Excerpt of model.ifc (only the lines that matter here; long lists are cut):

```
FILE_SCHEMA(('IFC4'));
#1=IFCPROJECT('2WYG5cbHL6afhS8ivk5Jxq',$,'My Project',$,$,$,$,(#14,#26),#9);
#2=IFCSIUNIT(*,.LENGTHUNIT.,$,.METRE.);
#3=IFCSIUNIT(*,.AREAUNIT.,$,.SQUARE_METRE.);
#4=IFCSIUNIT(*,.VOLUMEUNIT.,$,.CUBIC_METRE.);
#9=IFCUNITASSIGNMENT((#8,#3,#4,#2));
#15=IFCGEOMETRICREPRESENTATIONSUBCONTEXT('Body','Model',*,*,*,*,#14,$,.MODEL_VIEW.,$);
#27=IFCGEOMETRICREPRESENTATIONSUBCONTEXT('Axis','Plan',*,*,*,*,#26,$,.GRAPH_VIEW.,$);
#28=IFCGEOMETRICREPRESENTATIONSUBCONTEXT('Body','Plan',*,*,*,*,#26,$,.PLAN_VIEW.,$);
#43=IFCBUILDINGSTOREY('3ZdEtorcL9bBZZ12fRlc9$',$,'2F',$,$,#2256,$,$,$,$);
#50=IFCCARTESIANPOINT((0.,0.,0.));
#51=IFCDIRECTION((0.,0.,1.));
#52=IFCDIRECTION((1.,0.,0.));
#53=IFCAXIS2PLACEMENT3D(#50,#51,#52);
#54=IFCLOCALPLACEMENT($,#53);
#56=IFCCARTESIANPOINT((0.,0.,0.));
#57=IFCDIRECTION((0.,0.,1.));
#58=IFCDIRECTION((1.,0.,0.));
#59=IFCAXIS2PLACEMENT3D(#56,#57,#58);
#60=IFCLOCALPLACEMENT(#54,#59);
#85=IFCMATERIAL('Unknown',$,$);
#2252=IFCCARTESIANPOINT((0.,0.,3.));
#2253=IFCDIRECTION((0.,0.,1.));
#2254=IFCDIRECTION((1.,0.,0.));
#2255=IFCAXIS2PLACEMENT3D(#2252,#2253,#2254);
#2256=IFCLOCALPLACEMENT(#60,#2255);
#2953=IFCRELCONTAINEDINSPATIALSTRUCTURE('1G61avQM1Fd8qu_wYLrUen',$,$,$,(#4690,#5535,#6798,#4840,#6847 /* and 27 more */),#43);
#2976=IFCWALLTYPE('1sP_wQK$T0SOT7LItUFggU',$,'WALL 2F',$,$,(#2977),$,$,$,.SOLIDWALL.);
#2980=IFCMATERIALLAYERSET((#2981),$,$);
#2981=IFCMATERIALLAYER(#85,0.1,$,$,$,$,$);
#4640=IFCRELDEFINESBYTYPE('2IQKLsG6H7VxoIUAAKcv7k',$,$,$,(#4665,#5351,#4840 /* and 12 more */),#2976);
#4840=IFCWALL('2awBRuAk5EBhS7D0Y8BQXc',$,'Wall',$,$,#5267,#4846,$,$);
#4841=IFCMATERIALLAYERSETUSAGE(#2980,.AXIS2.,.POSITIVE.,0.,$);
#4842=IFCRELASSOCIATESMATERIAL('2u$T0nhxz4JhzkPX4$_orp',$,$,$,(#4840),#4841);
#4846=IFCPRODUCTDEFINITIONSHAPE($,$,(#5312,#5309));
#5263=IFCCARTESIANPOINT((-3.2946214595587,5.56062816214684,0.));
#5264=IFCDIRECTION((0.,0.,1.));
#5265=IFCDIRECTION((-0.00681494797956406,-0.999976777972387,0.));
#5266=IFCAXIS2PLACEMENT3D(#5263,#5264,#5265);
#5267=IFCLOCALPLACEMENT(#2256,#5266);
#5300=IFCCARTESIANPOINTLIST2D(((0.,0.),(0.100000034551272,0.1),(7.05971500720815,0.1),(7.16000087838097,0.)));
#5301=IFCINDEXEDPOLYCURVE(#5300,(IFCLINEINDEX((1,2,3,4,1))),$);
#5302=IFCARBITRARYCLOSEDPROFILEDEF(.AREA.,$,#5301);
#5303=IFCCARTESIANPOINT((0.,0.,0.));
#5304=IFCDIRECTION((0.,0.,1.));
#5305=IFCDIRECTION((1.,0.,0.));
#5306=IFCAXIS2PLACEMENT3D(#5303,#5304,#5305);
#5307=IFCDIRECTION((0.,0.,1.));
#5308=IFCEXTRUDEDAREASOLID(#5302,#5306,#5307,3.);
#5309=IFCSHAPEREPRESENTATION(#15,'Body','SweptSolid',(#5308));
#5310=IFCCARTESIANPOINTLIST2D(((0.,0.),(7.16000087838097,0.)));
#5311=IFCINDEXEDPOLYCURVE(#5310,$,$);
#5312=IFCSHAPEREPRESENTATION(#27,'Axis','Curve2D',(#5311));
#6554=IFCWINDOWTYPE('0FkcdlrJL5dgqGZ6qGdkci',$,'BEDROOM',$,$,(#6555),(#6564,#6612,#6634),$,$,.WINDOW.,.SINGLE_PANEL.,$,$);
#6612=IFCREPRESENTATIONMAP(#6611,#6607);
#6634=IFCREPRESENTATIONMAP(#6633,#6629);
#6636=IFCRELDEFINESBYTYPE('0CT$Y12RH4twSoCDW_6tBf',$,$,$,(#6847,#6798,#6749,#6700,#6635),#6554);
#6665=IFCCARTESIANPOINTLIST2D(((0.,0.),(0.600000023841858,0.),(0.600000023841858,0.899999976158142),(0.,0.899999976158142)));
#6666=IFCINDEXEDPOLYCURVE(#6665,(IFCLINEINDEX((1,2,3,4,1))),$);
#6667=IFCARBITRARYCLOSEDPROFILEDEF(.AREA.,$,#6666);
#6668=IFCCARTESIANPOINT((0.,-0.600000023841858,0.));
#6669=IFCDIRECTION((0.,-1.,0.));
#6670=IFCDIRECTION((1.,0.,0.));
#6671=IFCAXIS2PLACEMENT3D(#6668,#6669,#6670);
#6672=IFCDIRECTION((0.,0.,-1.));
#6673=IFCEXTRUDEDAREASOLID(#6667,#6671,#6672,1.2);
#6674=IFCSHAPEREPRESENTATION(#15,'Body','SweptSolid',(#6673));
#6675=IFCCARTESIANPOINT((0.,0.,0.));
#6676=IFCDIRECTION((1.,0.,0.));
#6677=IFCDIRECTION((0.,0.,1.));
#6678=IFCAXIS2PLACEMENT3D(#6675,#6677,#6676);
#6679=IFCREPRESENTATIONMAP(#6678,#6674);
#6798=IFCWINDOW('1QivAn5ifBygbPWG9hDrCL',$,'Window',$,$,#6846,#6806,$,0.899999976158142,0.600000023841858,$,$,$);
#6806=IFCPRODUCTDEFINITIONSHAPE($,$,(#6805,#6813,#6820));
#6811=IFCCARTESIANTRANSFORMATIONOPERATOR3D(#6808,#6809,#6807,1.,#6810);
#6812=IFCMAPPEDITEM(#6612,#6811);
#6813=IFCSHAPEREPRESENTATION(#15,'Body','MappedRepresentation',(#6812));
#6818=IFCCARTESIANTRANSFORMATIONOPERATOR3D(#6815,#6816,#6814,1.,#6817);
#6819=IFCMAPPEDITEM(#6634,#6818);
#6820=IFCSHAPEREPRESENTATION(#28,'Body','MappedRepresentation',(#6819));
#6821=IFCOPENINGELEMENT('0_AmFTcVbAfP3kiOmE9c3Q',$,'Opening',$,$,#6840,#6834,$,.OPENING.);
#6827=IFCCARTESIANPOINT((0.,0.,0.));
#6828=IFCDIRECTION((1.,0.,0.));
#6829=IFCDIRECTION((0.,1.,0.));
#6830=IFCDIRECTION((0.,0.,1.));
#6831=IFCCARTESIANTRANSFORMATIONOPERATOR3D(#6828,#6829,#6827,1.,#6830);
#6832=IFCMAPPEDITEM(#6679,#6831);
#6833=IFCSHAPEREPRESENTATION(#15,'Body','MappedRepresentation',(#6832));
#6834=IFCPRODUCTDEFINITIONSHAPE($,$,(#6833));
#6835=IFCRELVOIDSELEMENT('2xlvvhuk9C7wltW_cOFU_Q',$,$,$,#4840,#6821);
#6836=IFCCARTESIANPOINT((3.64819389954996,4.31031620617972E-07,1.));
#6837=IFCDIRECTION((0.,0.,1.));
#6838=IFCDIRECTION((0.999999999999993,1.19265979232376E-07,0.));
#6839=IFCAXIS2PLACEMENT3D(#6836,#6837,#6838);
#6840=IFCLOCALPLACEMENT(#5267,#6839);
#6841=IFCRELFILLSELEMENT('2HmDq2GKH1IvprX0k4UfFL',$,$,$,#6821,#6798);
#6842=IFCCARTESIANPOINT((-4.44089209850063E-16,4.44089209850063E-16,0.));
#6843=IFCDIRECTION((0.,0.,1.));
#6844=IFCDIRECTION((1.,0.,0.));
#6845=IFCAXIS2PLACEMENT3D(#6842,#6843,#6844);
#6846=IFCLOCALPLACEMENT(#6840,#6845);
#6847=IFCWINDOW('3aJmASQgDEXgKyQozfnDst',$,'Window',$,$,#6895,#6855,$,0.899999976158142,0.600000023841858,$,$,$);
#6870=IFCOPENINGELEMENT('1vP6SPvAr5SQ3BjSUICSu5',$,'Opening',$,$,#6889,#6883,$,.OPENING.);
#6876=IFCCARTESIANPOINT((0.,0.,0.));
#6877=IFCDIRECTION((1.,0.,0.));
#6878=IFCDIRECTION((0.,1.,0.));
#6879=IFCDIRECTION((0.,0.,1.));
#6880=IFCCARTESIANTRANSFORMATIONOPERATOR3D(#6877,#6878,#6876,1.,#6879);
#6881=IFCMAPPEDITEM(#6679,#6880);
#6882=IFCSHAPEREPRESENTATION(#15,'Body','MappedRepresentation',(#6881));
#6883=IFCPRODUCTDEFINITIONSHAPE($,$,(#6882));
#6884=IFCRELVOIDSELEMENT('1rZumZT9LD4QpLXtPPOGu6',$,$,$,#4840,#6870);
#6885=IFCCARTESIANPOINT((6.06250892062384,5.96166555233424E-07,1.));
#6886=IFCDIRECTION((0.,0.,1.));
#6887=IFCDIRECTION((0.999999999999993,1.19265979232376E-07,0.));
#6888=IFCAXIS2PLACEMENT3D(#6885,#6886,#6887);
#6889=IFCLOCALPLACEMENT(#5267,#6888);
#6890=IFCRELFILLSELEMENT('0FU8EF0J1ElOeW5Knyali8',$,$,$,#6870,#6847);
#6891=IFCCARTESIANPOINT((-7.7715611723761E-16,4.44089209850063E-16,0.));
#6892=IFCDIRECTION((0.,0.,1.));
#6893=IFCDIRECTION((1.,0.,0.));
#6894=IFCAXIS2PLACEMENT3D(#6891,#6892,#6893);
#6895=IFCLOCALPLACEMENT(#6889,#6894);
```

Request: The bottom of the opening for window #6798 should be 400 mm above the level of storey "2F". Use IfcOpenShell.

```python
import numpy as np
import ifcopenshell
import ifcopenshell.api.geometry
import ifcopenshell.geom
import ifcopenshell.util.element
import ifcopenshell.util.placement
import ifcopenshell.util.shape
import ifcopenshell.util.unit

model = ifcopenshell.open("model.ifc")
unit_scale = ifcopenshell.util.unit.calculate_unit_scale(model)

window = model.by_id(6798)
opening = window.FillsVoids[0].RelatingOpeningElement
storey = ifcopenshell.util.element.get_container(window, ifc_class="IfcBuildingStorey")
level = ifcopenshell.util.placement.get_local_placement(storey.ObjectPlacement)[2, 3]

# The opening's origin need not be at the sill, so measure its lowest point.
shape = ifcopenshell.geom.create_shape(ifcopenshell.geom.settings(), opening)
bottom = ifcopenshell.util.shape.get_shape_bottom_elevation(shape, shape.geometry) / unit_scale
dz = level + 0.4 / unit_scale - bottom

shift = np.array([0.0, 0.0, dz])
# The window is placed relative to its opening, so it follows when the opening moves.
matrix = ifcopenshell.util.placement.get_local_placement(opening.ObjectPlacement)
matrix[:3, 3] += shift
ifcopenshell.api.geometry.edit_object_placement(
    model, product=opening, matrix=matrix, is_si=False, should_transform_children=True
)

print(f"moved by {dz * unit_scale:+.3f} m")

model.write("model_rev.ifc")
```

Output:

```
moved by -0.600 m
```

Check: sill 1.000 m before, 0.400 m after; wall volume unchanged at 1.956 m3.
